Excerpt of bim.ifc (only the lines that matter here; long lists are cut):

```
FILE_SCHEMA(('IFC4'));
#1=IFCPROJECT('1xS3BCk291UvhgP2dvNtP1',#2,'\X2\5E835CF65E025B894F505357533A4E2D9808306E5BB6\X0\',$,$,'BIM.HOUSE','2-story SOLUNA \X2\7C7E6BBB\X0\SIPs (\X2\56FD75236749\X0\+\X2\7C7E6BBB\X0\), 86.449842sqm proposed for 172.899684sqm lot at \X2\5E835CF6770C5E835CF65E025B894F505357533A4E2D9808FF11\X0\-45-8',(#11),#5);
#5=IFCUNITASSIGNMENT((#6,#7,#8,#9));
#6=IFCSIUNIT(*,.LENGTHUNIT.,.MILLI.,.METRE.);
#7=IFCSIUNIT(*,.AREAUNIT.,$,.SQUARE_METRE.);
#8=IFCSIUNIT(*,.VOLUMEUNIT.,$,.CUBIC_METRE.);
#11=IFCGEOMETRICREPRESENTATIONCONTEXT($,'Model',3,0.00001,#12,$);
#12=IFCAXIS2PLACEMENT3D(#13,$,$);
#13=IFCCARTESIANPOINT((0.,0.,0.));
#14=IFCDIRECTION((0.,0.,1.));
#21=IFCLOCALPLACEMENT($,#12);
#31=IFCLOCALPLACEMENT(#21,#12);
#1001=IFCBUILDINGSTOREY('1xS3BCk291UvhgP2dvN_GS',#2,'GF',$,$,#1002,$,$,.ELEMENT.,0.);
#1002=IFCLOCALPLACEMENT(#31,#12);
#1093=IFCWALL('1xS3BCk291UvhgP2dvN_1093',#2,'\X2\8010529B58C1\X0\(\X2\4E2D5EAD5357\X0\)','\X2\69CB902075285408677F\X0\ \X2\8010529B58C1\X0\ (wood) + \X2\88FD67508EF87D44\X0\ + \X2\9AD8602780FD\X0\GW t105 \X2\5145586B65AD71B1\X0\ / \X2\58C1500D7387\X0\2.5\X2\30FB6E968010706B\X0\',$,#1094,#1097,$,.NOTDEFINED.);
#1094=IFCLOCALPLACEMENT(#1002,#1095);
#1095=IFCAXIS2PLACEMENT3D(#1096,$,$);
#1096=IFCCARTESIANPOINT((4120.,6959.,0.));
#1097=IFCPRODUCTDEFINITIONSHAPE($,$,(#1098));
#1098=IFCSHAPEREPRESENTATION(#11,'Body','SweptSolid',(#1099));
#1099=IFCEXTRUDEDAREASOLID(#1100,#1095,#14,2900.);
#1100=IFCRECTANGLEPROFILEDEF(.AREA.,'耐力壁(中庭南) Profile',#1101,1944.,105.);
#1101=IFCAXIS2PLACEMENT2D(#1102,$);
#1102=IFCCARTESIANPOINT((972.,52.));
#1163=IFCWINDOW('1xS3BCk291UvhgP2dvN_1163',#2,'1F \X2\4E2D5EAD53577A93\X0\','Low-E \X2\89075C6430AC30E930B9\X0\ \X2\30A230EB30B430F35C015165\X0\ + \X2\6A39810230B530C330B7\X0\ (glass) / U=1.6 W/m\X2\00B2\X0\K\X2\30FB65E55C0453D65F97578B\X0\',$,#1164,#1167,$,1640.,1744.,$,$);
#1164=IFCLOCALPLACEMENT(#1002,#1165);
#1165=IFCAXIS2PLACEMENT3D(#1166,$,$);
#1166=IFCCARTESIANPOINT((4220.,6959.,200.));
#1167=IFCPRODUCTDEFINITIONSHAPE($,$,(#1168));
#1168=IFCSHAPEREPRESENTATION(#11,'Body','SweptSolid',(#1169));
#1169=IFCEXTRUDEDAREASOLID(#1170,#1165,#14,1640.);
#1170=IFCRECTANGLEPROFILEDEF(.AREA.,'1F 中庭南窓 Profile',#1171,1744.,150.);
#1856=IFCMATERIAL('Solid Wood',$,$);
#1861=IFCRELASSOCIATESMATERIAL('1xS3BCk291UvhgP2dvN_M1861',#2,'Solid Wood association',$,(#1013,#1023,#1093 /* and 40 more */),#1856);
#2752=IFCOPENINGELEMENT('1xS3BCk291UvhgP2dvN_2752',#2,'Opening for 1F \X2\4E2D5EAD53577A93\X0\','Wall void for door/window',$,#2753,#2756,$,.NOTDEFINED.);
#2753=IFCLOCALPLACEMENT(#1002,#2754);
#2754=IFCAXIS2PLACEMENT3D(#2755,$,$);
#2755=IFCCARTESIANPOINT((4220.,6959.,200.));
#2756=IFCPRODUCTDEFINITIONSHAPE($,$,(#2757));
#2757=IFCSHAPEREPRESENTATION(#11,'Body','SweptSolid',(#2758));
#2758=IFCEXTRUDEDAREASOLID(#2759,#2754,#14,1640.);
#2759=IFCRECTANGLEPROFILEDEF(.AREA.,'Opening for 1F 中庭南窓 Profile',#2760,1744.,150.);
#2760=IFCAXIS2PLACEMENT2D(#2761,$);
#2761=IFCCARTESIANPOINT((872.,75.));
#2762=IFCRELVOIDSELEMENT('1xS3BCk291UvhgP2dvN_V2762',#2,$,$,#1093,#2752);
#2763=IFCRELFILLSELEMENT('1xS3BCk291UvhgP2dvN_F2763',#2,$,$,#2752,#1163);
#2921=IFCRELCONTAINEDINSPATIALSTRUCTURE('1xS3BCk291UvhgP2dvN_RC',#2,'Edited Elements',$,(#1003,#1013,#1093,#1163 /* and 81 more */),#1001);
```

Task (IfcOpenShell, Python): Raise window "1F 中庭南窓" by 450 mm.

```python
import numpy as np
import ifcopenshell
import ifcopenshell.api.geometry
import ifcopenshell.util.placement
import ifcopenshell.util.unit

model = ifcopenshell.open("bim.ifc")
unit_scale = ifcopenshell.util.unit.calculate_unit_scale(model)

window = model.by_guid("1xS3BCk291UvhgP2dvN_1163")
opening = window.FillsVoids[0].RelatingOpeningElement
dz = 0.45 / unit_scale

shift = np.array([0.0, 0.0, dz])
# The window is not placed relative to its opening, so move both.
for product in (opening, window):
    matrix = ifcopenshell.util.placement.get_local_placement(product.ObjectPlacement)
    matrix[:3, 3] += shift
    ifcopenshell.api.geometry.edit_object_placement(model, product=product, matrix=matrix, is_si=False)

print(f"moved by {dz * unit_scale:+.3f} m")

model.write("bim_updated.ifc")
```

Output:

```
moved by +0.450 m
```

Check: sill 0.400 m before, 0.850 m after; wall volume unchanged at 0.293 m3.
